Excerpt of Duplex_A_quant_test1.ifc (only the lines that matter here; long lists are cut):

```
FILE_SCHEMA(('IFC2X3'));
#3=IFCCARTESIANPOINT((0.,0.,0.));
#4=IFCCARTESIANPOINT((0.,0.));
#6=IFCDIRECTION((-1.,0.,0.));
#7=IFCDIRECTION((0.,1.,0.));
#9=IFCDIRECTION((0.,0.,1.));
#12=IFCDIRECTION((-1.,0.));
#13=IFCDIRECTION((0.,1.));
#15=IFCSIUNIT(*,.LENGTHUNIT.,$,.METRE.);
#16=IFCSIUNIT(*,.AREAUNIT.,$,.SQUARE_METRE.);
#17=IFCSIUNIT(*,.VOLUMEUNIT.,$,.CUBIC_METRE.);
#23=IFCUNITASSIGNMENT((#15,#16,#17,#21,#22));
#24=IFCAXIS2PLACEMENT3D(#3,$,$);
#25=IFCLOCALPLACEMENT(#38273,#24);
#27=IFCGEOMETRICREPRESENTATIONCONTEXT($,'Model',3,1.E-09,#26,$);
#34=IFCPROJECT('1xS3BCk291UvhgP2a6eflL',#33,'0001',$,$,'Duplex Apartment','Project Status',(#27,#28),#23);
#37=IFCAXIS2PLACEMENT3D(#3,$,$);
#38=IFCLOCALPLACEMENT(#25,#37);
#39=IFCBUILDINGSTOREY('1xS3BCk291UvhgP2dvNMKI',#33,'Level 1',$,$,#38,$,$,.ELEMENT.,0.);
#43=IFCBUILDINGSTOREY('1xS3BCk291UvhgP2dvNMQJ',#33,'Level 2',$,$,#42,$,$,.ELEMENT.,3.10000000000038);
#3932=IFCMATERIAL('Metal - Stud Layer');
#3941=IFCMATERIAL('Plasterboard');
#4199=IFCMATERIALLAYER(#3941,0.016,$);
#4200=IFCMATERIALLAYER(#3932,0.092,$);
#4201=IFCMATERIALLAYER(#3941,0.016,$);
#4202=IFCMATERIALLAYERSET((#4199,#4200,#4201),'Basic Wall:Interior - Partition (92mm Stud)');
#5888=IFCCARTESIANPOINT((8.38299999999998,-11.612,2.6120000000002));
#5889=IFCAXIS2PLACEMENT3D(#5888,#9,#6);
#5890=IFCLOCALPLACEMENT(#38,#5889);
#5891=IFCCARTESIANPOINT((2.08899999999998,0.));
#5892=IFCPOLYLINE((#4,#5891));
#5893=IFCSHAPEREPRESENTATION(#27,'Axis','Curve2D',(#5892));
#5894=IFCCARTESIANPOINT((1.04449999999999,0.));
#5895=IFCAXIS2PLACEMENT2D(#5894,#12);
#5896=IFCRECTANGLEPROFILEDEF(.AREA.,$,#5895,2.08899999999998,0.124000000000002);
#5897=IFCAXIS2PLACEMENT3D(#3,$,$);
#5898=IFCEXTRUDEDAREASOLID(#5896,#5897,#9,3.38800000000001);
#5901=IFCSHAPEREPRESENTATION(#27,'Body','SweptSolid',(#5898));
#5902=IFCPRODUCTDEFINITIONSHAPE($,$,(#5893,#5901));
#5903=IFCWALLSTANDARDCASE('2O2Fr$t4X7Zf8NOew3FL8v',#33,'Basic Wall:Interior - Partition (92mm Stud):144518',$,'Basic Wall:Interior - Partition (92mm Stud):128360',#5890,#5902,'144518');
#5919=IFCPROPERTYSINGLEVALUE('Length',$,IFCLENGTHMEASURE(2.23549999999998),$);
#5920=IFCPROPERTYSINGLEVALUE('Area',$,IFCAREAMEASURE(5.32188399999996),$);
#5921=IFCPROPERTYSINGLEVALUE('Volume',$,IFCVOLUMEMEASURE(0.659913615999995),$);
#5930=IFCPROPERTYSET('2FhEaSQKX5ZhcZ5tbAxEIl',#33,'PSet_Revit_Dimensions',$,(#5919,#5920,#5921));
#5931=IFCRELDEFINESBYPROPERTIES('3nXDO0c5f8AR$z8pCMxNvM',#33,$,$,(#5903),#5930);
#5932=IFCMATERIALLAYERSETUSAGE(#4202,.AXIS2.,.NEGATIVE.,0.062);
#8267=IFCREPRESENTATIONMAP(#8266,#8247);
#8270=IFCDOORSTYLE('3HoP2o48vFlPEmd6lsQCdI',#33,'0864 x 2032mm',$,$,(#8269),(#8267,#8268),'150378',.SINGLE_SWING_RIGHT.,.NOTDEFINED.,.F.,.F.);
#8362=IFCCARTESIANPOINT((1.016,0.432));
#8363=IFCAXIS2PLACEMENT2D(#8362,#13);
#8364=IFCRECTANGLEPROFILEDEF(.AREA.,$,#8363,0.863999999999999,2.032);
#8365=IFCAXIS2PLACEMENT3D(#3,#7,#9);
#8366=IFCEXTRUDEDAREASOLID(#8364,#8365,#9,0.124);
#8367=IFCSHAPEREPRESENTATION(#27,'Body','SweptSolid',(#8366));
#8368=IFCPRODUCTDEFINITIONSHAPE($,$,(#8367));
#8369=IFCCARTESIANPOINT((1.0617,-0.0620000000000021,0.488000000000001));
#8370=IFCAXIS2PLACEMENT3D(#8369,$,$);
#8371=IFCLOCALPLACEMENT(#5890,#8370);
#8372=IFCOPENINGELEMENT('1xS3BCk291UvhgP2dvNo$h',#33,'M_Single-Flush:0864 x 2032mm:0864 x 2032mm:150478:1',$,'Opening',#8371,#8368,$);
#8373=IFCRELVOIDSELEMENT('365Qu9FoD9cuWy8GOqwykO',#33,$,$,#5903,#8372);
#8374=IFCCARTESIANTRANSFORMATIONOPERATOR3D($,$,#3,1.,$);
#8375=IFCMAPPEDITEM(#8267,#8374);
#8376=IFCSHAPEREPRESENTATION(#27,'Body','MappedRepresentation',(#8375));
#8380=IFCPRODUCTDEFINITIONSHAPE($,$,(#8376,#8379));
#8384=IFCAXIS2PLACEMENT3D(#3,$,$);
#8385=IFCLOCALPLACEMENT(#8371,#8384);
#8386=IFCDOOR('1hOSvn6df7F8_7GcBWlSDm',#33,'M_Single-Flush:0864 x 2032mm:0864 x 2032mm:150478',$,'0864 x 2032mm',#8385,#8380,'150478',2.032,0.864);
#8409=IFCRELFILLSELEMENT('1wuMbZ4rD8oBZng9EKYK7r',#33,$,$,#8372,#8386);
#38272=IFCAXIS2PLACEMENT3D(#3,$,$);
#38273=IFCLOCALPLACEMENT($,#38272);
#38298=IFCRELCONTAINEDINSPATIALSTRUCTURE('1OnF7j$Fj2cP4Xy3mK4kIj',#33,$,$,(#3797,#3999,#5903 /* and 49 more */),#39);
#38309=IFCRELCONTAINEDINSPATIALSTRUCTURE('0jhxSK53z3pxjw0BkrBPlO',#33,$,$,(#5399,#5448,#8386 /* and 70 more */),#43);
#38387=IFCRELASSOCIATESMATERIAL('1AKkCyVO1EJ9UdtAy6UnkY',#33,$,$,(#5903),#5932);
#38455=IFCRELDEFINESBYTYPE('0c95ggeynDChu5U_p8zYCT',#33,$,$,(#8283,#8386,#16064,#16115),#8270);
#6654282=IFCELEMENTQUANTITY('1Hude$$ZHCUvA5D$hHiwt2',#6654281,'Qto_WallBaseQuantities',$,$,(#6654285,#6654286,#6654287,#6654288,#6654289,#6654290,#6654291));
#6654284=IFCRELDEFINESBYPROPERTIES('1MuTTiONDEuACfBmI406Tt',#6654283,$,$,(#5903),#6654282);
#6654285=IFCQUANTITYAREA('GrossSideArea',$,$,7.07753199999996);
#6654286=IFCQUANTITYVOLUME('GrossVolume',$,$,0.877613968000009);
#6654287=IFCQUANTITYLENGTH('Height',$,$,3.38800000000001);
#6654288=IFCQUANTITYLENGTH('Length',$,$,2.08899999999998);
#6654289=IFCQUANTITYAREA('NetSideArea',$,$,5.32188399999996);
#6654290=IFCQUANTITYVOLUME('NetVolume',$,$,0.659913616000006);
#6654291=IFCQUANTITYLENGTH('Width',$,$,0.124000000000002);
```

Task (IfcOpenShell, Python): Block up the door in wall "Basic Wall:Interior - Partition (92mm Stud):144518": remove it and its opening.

```python
import ifcopenshell
import ifcopenshell.api.feature
import ifcopenshell.api.pset
import ifcopenshell.api.root
import ifcopenshell.geom
import ifcopenshell.util.element
import ifcopenshell.util.shape
import ifcopenshell.util.unit

model = ifcopenshell.open("Duplex_A_quant_test1.ifc")
area_scale = ifcopenshell.util.unit.calculate_unit_scale(model, "AREAUNIT")
volume_scale = ifcopenshell.util.unit.calculate_unit_scale(model, "VOLUMEUNIT")
settings = ifcopenshell.geom.settings()


def volume(element):
    """Net volume in cubic metres, openings subtracted."""
    shape = ifcopenshell.geom.create_shape(settings, element)
    return ifcopenshell.util.shape.get_volume(shape.geometry)


door = model.by_guid("1hOSvn6df7F8_7GcBWlSDm")
opening = door.FillsVoids[0].RelatingOpeningElement
wall = opening.VoidsElements[0].RelatingBuildingElement
before = volume(wall)

ifcopenshell.api.root.remove_product(model, product=door)
ifcopenshell.api.feature.remove_feature(model, feature=opening)

after = volume(wall)
thickness = 0.124  # wall thickness in metres

# Update the wall's stored quantities.
pset = model.by_id(ifcopenshell.util.element.get_pset(wall, "PSet_Revit_Dimensions", should_inherit=False)["id"])
ifcopenshell.api.pset.edit_pset(model, pset=pset, properties={
    "Area": model.create_entity("IfcAreaMeasure", after / thickness / area_scale),
    "Volume": model.create_entity("IfcVolumeMeasure", after / volume_scale),
})
qto = model.by_id(ifcopenshell.util.element.get_pset(wall, "Qto_WallBaseQuantities", should_inherit=False)["id"])
ifcopenshell.api.pset.edit_qto(model, qto=qto, properties={
    "NetSideArea": after / thickness / area_scale,
    "NetVolume": after / volume_scale,
})

print(f"wall volume {before:.3f} -> {after:.3f} m3")

model.write("Duplex_A_quant_test1-out.ifc")
```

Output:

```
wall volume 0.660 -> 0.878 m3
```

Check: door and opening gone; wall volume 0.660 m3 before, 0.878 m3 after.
